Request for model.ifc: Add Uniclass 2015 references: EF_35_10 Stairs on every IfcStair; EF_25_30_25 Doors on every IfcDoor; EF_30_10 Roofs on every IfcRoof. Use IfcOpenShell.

First a look at what the model holds.

```python
import ifcopenshell

model = ifcopenshell.open("model.ifc")
print(model.schema)
print("classifications:", [c.Name for c in model.by_type("IfcClassification")])
for ifc_class in ("IfcDoor", "IfcRoof", "IfcStair", "IfcWall", "IfcWindow"):
    print(ifc_class, len(model.by_type(ifc_class)))
```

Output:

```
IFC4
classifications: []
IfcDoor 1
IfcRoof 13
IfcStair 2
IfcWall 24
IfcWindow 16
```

```python
import ifcopenshell
import ifcopenshell.api.classification

model = ifcopenshell.open("model.ifc")

system = ifcopenshell.api.classification.add_classification(model, classification="Uniclass 2015")

codes = {
    "IfcStair": ("EF_35_10", "Stairs"),
    "IfcDoor": ("EF_25_30_25", "Doors"),
    "IfcRoof": ("EF_30_10", "Roofs"),
}
for ifc_class, (code, name) in codes.items():
    products = model.by_type(ifc_class)
    ifcopenshell.api.classification.add_reference(
        model, products=products, classification=system, identification=code, name=name
    )
    print(code, len(products))

model.write("model_edited.ifc")
```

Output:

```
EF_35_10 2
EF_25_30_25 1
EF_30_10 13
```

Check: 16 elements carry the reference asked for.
